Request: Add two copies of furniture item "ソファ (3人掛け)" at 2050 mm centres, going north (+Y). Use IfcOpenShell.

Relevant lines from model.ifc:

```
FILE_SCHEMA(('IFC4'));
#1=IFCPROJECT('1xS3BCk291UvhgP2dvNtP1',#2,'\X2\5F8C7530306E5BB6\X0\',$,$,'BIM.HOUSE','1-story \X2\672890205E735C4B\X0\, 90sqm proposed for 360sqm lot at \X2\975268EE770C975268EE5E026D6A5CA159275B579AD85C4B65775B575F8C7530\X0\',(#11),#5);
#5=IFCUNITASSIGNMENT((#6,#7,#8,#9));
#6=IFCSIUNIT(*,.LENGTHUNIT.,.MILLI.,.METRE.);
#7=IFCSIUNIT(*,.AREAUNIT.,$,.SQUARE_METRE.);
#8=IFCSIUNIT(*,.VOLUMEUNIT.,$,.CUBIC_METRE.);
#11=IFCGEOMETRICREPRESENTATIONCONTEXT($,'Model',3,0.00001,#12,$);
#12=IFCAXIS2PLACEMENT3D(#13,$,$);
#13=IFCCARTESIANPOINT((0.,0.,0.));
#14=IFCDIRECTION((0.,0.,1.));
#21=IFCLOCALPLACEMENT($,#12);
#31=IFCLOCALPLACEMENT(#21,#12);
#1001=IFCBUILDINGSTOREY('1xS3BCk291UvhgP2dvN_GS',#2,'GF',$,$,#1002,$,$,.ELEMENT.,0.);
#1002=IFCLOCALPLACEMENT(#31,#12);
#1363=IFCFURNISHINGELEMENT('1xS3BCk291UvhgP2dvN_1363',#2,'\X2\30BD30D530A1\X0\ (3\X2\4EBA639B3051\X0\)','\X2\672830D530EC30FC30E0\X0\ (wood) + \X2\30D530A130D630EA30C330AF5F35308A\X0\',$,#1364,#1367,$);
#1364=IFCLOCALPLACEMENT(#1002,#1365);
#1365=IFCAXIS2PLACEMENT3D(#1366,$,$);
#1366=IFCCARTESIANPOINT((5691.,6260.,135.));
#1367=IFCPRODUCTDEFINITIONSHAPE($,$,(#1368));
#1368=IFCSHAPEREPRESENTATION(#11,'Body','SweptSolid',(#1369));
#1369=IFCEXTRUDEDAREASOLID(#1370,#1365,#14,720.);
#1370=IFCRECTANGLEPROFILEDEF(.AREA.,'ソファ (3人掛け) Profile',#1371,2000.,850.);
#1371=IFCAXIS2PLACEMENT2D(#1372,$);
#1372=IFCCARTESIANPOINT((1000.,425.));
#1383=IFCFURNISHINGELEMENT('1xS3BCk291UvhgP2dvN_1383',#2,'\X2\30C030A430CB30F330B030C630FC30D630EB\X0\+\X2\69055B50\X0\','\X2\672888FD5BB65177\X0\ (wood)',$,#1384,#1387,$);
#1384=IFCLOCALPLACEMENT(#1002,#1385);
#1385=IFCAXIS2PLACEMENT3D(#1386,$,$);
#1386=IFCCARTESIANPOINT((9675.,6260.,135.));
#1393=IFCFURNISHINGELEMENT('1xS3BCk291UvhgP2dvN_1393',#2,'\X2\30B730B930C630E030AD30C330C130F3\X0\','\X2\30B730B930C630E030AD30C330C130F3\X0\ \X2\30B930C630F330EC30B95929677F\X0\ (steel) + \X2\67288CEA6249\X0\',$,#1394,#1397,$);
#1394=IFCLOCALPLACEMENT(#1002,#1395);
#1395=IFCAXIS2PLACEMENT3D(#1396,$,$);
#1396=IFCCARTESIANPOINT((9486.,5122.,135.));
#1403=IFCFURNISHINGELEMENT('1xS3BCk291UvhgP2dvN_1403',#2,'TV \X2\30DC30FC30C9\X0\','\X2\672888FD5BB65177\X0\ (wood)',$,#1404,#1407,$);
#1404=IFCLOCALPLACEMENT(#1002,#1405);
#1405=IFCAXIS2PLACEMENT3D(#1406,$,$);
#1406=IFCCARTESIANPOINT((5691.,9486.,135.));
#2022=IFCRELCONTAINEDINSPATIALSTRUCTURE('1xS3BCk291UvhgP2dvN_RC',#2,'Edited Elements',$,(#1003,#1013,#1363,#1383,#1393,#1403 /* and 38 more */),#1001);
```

```python
import numpy as np
import ifcopenshell
import ifcopenshell.api.geometry
import ifcopenshell.api.root
import ifcopenshell.util.element
import ifcopenshell.util.placement
import ifcopenshell.util.unit

model = ifcopenshell.open("model.ifc")
unit_scale = ifcopenshell.util.unit.calculate_unit_scale(model)


def reuse_history(source, copy):
    """copy_class also copies each property set's owner history, people and application; keep the originals."""
    for rel in copy.IsDefinedBy:
        if rel.is_a("IfcRelDefinesByProperties") and (history := rel.RelatingPropertyDefinition.OwnerHistory):
            rel.RelatingPropertyDefinition.OwnerHistory = source.OwnerHistory
            ifcopenshell.util.element.remove_deep2(model, history)


source = model.by_guid("1xS3BCk291UvhgP2dvN_1363")
base = ifcopenshell.util.placement.get_local_placement(source.ObjectPlacement)
step = np.array([0.0, 1.0, 0.0]) * 2.05 / unit_scale

for i in range(1, 3):
    copy = ifcopenshell.api.root.copy_class(model, product=source)
    copy.Representation = ifcopenshell.util.element.copy_deep(
        model, source.Representation, exclude=["IfcGeometricRepresentationContext", "IfcRepresentationMap"]
    )
    reuse_history(source, copy)
    matrix = base.copy()
    matrix[:3, 3] += i * step
    print("added at", matrix[:3, 3].round(3) + 0.0)
    ifcopenshell.api.geometry.edit_object_placement(model, product=copy, matrix=matrix, is_si=False)

model.write("model-out.ifc")
```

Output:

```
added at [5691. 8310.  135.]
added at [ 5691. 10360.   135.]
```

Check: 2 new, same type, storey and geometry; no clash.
